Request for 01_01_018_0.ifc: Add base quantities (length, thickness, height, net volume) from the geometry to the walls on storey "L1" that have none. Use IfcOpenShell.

First a look at what the model holds.

```python
import ifcopenshell
import ifcopenshell.util.element
import ifcopenshell.util.unit

model = ifcopenshell.open("01_01_018_0.ifc")
print(model.schema)
for unit_type in ("LENGTHUNIT", "AREAUNIT", "VOLUMEUNIT"):
    print(unit_type, ifcopenshell.util.unit.calculate_unit_scale(model, unit_type))
storey = next(s for s in model.by_type("IfcBuildingStorey") if s.Name == "L1")
walls = [e for e in ifcopenshell.util.element.get_decomposition(storey) if e.is_a("IfcWall")]
for e in sorted(walls, key=lambda e: e.id()):
    print(e.id(), e.is_a(), e.Name, list(ifcopenshell.util.element.get_psets(e, qtos_only=True)), sep=" | ")
```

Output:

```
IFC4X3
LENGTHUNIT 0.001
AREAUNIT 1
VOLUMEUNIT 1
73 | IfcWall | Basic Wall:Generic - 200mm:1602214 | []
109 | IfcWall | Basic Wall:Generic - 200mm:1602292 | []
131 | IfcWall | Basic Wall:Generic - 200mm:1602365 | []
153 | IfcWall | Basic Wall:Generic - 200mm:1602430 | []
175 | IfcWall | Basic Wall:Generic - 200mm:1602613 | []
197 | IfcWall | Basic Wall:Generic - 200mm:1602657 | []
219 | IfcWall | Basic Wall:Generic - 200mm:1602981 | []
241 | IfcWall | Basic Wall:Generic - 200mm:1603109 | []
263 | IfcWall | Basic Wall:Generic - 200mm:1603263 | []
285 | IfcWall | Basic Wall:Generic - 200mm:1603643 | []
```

```python
import ifcopenshell
import ifcopenshell.api.pset
import ifcopenshell.geom
import ifcopenshell.util.element
import ifcopenshell.util.shape
import ifcopenshell.util.unit

model = ifcopenshell.open("01_01_018_0.ifc")
unit_scale = ifcopenshell.util.unit.calculate_unit_scale(model)
volume_scale = ifcopenshell.util.unit.calculate_unit_scale(model, "VOLUMEUNIT")
settings = ifcopenshell.geom.settings()

storey = next(s for s in model.by_type("IfcBuildingStorey") if s.Name == "L1")
walls = [e for e in ifcopenshell.util.element.get_decomposition(storey) if e.is_a("IfcWall")]

for e in sorted(walls, key=lambda e: e.id()):
    if ifcopenshell.util.element.get_psets(e, qtos_only=True, should_inherit=False):
        continue
    # Geometry comes back in metres, in the element's own axes.
    shape = ifcopenshell.geom.create_shape(settings, e)
    values = {
        "Length": ifcopenshell.util.shape.get_x(shape.geometry) / unit_scale,
        "Width": ifcopenshell.util.shape.get_y(shape.geometry) / unit_scale,
        "Height": ifcopenshell.util.shape.get_z(shape.geometry) / unit_scale,
        "NetVolume": ifcopenshell.util.shape.get_volume(shape.geometry) / volume_scale,
    }
    qto = ifcopenshell.api.pset.add_qto(model, product=e, name="Qto_WallBaseQuantities")
    ifcopenshell.api.pset.edit_qto(model, qto=qto, properties=values)
    print(e.id(), {k: round(v, 3) for k, v in values.items()})

model.write("01_01_018_0_rev.ifc")
```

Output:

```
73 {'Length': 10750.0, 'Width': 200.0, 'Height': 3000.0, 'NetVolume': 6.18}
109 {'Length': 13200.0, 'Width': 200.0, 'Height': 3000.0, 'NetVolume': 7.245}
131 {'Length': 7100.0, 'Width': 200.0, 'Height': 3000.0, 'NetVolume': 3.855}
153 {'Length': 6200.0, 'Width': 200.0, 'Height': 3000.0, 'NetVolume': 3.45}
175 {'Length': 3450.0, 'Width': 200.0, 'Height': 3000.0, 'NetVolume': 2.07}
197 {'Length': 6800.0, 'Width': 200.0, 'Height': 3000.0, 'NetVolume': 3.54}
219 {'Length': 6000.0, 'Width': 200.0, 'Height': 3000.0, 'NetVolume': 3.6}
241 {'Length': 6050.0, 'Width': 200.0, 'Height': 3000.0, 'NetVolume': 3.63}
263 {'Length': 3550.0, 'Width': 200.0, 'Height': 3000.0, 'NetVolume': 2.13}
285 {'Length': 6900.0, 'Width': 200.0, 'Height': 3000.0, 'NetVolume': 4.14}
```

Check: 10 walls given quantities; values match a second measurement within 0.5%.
